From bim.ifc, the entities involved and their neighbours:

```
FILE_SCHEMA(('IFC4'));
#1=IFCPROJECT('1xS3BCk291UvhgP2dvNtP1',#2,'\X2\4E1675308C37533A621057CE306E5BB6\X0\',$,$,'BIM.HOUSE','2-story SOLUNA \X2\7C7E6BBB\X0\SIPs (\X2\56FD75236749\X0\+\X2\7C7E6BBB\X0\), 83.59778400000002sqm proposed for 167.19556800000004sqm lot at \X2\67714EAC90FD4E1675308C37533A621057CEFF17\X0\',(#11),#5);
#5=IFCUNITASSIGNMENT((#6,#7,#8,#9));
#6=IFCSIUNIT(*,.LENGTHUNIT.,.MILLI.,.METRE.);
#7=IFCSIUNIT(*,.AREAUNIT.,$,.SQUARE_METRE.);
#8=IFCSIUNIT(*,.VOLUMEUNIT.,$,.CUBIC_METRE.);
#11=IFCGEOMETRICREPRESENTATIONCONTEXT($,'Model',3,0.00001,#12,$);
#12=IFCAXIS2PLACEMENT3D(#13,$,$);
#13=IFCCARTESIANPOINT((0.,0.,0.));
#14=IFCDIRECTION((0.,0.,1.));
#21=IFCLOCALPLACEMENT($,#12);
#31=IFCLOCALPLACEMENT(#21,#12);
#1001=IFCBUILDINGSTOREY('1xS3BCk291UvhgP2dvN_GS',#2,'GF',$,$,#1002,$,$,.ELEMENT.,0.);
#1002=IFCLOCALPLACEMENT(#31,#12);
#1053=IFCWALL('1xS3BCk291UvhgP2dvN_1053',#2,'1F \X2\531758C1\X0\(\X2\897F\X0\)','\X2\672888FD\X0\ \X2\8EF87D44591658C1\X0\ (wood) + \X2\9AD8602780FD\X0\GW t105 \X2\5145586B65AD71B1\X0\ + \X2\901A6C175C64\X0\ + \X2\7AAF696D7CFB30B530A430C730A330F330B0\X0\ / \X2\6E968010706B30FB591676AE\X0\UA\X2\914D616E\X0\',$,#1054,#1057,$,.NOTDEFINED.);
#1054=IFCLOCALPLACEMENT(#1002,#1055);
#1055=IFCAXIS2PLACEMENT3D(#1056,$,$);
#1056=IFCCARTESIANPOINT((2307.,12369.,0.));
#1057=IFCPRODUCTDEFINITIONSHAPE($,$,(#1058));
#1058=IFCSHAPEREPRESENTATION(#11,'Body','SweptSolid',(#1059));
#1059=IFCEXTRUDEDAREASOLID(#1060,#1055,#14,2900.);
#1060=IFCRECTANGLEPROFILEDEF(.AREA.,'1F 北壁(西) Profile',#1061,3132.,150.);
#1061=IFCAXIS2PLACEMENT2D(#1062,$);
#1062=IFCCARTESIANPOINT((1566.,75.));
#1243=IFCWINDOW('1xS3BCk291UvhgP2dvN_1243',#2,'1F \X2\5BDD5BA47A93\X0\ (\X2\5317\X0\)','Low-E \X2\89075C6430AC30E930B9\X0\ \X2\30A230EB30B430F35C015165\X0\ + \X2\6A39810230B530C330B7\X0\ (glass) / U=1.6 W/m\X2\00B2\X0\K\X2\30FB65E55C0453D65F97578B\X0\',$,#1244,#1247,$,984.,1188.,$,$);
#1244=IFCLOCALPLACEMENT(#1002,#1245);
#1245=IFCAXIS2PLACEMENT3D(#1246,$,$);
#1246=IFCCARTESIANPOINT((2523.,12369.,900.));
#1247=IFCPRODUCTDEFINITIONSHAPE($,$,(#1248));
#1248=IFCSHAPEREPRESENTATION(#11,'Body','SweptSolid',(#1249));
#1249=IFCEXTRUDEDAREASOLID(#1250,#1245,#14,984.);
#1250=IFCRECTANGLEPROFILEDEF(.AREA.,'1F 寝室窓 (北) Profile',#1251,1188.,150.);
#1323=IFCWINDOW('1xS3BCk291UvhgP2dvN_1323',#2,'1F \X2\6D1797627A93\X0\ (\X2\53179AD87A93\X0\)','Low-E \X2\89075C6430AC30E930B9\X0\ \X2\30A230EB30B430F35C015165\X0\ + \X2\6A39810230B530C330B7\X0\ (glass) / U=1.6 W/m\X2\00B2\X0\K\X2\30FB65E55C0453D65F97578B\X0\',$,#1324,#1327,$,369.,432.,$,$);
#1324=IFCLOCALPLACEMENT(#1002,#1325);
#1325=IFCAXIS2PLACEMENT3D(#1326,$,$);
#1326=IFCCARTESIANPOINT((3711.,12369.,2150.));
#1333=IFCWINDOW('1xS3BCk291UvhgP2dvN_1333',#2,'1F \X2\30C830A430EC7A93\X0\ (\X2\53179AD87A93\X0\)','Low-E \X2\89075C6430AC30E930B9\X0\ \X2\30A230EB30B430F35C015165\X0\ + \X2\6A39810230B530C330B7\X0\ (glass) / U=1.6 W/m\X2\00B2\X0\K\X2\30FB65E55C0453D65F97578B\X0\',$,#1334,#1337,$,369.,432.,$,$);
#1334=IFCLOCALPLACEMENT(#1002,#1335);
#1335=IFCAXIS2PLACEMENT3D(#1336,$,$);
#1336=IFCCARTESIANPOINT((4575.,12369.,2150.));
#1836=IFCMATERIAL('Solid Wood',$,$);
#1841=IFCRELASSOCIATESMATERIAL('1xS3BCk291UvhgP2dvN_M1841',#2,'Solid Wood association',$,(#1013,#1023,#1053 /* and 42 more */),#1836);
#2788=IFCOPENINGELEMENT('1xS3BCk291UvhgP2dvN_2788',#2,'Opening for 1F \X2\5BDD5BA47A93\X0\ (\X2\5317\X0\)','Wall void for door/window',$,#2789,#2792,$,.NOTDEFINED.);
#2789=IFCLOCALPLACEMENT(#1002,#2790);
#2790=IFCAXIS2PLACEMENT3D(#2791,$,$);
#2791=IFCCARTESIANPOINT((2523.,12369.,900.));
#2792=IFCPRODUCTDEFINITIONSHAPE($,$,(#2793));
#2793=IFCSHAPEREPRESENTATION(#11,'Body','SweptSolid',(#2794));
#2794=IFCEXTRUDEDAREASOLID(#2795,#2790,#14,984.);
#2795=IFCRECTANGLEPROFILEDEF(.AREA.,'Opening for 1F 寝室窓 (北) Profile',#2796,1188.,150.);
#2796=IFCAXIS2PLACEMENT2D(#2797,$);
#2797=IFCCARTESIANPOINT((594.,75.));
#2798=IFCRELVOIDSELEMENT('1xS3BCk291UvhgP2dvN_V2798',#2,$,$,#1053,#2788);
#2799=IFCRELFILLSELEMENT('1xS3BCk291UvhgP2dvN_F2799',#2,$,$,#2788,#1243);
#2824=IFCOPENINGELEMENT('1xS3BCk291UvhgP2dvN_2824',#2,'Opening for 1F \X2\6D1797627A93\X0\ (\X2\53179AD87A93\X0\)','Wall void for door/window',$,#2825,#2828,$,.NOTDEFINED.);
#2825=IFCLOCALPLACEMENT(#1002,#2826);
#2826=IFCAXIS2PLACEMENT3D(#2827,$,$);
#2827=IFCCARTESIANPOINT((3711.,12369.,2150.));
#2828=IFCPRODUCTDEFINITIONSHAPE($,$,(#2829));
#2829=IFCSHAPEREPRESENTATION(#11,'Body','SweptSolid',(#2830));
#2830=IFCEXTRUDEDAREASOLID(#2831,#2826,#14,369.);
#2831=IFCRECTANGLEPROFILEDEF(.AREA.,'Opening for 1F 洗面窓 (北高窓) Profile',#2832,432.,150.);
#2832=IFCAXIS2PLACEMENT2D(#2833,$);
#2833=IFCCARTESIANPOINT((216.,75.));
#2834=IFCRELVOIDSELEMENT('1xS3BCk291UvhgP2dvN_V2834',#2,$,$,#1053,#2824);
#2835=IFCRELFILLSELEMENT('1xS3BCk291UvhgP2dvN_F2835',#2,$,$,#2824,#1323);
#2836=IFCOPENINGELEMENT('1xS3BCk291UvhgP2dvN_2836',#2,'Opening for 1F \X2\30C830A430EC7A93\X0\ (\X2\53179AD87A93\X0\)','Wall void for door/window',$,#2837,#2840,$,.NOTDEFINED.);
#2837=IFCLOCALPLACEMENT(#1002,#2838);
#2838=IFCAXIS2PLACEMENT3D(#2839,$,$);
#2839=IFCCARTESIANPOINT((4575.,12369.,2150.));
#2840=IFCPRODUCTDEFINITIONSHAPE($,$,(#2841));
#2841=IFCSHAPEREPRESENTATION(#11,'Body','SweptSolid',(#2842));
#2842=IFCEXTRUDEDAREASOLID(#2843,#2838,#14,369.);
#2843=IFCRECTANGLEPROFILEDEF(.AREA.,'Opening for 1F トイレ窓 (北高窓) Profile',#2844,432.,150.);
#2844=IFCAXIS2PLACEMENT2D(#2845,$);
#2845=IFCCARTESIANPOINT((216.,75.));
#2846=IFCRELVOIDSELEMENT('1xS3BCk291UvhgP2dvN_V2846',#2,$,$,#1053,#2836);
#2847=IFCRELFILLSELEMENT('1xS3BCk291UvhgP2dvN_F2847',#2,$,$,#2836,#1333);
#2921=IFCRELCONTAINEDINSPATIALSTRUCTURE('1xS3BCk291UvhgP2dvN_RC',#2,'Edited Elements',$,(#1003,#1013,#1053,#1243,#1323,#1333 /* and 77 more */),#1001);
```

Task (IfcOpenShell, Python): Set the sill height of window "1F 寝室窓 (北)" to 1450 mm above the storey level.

```python
import numpy as np
import ifcopenshell
import ifcopenshell.api.geometry
import ifcopenshell.geom
import ifcopenshell.util.element
import ifcopenshell.util.placement
import ifcopenshell.util.shape
import ifcopenshell.util.unit

model = ifcopenshell.open("bim.ifc")
unit_scale = ifcopenshell.util.unit.calculate_unit_scale(model)

window = model.by_guid("1xS3BCk291UvhgP2dvN_1243")
opening = window.FillsVoids[0].RelatingOpeningElement
storey = ifcopenshell.util.element.get_container(window, ifc_class="IfcBuildingStorey")
level = ifcopenshell.util.placement.get_local_placement(storey.ObjectPlacement)[2, 3]

# The opening's origin need not be at the sill, so measure its lowest point.
shape = ifcopenshell.geom.create_shape(ifcopenshell.geom.settings(), opening)
bottom = ifcopenshell.util.shape.get_shape_bottom_elevation(shape, shape.geometry) / unit_scale
dz = level + 1450.0 - bottom

shift = np.array([0.0, 0.0, dz])
# The window is not placed relative to its opening, so move both.
for product in (opening, window):
    matrix = ifcopenshell.util.placement.get_local_placement(product.ObjectPlacement)
    matrix[:3, 3] += shift
    ifcopenshell.api.geometry.edit_object_placement(model, product=product, matrix=matrix, is_si=False)

print(f"moved by {dz * unit_scale:+.3f} m")

model.write("bim-out.ifc")
```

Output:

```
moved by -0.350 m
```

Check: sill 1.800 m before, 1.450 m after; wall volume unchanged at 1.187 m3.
